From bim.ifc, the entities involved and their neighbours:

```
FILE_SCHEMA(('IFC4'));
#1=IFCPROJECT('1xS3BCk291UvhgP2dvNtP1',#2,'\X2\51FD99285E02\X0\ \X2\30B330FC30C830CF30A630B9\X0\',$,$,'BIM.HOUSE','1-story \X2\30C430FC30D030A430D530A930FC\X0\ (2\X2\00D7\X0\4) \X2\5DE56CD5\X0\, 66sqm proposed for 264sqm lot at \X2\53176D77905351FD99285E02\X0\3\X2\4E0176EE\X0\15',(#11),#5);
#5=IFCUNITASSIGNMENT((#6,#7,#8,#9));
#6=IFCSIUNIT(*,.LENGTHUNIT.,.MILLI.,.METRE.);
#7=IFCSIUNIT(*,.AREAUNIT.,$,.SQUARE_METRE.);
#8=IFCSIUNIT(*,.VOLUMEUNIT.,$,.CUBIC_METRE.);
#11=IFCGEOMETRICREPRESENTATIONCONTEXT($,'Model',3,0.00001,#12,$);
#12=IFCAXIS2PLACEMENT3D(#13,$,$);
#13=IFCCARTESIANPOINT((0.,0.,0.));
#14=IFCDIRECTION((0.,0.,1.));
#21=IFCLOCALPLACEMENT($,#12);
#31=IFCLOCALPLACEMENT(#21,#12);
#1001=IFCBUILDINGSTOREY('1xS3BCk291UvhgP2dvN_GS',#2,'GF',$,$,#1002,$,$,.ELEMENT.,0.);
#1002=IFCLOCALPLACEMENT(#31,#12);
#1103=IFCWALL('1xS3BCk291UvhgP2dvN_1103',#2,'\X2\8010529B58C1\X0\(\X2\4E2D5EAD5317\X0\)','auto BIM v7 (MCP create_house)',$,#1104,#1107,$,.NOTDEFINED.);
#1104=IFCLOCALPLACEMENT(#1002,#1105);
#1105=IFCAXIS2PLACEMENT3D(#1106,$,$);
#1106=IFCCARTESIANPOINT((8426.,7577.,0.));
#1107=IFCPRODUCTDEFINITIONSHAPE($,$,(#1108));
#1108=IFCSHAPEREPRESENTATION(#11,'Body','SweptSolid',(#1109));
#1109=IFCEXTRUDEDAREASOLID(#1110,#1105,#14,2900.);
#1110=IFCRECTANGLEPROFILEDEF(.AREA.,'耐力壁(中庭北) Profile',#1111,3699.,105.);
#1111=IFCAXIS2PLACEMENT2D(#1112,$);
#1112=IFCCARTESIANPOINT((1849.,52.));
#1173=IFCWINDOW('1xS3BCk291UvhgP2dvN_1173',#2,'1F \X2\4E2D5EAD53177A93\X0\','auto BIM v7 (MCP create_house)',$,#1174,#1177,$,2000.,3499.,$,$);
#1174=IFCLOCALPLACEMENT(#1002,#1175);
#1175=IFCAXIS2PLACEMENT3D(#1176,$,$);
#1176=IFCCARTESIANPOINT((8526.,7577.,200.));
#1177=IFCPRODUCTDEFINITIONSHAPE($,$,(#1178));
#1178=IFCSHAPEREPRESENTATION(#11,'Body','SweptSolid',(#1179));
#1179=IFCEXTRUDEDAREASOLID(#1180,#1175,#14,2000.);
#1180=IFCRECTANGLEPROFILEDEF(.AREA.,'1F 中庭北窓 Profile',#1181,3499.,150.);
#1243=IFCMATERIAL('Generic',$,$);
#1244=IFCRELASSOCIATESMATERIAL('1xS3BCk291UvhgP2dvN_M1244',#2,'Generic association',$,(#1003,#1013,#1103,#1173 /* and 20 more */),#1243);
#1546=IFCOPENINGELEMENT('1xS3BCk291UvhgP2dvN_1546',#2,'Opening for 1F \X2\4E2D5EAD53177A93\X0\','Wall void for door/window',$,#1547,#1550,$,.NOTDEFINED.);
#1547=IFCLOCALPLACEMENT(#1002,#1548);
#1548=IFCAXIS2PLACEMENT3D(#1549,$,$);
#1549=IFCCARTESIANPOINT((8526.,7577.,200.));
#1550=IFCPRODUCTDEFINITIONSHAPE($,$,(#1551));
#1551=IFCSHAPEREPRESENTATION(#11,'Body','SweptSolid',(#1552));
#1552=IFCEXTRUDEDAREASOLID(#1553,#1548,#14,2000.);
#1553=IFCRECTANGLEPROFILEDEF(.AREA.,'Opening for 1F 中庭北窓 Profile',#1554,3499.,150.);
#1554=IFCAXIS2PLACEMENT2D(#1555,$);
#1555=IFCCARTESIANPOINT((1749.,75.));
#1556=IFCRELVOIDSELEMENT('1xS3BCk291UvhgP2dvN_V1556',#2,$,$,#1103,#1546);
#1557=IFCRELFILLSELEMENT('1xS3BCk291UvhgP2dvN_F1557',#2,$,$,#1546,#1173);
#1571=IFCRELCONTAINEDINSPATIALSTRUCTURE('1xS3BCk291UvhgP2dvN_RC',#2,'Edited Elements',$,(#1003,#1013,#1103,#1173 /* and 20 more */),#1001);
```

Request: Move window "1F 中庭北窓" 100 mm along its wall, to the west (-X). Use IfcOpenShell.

```python
import ifcopenshell
import ifcopenshell.api.geometry
import ifcopenshell.util.placement
import ifcopenshell.util.unit

model = ifcopenshell.open("bim.ifc")
unit_scale = ifcopenshell.util.unit.calculate_unit_scale(model)

window = model.by_guid("1xS3BCk291UvhgP2dvN_1173")
opening = window.FillsVoids[0].RelatingOpeningElement
wall = opening.VoidsElements[0].RelatingBuildingElement

wall_matrix = ifcopenshell.util.placement.get_local_placement(wall.ObjectPlacement)
shift = wall_matrix[:3, 0] * -0.1 / unit_scale
before = ifcopenshell.util.placement.get_local_placement(window.ObjectPlacement)[:3, 3].copy()

# The window is not placed relative to its opening, so move both.
for product in (opening, window):
    matrix = ifcopenshell.util.placement.get_local_placement(product.ObjectPlacement)
    matrix[:3, 3] += shift
    ifcopenshell.api.geometry.edit_object_placement(model, product=product, matrix=matrix, is_si=False)

after = ifcopenshell.util.placement.get_local_placement(window.ObjectPlacement)[:3, 3]
print("window moved by", (after - before).round(3) + 0.0)

model.write("bim_updated.ifc")
```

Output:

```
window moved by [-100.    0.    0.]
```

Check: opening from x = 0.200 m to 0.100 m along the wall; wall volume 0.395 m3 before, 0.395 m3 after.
